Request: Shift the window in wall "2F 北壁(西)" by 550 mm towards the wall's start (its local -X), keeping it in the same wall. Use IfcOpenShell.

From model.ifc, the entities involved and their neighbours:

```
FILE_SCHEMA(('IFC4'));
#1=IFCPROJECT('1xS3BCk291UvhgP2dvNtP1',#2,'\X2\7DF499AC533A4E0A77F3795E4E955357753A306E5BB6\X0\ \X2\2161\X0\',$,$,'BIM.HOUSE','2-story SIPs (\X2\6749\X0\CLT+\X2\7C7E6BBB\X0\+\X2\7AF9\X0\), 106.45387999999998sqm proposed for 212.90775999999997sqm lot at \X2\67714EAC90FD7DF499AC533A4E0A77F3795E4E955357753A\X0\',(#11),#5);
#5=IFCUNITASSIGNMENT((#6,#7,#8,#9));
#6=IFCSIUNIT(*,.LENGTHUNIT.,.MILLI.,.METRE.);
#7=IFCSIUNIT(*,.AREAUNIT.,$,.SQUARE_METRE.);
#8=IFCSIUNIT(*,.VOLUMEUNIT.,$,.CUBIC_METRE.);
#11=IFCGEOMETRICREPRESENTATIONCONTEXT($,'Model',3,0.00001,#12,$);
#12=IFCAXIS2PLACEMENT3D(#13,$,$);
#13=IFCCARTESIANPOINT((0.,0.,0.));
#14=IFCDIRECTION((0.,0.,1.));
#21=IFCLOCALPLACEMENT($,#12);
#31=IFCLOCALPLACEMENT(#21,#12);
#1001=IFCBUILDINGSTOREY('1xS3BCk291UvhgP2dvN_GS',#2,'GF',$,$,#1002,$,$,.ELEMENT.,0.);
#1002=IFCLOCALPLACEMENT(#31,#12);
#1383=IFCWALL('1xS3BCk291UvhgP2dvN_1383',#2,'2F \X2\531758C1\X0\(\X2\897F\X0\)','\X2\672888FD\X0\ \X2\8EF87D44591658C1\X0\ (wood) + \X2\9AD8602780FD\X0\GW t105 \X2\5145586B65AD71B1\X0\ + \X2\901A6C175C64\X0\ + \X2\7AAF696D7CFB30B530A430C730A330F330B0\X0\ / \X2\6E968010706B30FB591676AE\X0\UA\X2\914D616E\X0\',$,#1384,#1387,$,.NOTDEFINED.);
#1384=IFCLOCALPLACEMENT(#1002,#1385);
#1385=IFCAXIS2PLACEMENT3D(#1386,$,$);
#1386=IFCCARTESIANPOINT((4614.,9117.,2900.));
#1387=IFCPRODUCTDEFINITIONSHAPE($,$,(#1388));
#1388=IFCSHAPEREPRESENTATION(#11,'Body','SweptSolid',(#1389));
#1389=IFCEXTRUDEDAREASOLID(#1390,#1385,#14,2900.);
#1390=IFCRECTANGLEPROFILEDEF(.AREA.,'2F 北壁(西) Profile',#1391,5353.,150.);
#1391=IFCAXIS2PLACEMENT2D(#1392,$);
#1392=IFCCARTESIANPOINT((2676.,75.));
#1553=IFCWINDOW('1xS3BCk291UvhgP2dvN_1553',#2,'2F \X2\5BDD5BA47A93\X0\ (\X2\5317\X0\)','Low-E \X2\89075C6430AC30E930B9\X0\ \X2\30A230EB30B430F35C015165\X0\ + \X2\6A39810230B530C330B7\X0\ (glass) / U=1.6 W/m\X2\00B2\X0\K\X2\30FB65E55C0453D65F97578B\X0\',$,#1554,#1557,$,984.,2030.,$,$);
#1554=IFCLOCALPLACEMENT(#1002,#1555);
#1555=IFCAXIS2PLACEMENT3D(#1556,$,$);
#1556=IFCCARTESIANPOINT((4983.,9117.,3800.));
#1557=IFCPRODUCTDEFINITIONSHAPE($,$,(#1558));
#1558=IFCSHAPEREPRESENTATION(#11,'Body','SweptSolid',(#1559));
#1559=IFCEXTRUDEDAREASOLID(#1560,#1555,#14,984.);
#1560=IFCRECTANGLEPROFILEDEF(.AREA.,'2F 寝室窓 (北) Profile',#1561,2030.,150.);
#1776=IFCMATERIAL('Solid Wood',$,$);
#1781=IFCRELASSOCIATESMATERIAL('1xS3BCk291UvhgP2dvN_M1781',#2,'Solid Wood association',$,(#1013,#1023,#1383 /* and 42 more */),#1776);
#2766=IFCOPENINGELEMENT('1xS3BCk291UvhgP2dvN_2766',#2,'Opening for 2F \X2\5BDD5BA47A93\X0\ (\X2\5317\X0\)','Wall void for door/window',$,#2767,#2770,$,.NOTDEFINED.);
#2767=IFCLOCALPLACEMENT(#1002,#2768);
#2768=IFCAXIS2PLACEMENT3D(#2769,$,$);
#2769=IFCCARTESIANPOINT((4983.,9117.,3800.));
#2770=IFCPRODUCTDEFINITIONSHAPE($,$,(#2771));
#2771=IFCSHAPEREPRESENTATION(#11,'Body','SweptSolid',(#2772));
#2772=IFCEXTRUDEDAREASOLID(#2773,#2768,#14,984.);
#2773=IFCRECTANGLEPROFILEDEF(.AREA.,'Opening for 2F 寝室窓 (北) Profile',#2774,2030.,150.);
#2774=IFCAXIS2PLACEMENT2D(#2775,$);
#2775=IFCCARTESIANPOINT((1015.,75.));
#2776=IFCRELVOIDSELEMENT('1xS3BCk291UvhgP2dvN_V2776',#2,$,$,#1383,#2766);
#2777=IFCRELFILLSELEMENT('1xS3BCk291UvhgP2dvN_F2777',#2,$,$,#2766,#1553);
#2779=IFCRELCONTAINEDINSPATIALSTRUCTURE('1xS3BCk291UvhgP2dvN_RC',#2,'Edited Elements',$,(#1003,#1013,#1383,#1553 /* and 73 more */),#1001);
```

```python
import ifcopenshell
import ifcopenshell.api.geometry
import ifcopenshell.util.placement
import ifcopenshell.util.unit

model = ifcopenshell.open("model.ifc")
unit_scale = ifcopenshell.util.unit.calculate_unit_scale(model)

window = model.by_id(1553)
opening = window.FillsVoids[0].RelatingOpeningElement
wall = opening.VoidsElements[0].RelatingBuildingElement

wall_matrix = ifcopenshell.util.placement.get_local_placement(wall.ObjectPlacement)
shift = wall_matrix[:3, 0] * -0.55 / unit_scale
before = ifcopenshell.util.placement.get_local_placement(window.ObjectPlacement)[:3, 3].copy()

# The window is not placed relative to its opening, so move both.
for product in (opening, window):
    matrix = ifcopenshell.util.placement.get_local_placement(product.ObjectPlacement)
    matrix[:3, 3] += shift
    ifcopenshell.api.geometry.edit_object_placement(model, product=product, matrix=matrix, is_si=False)

after = ifcopenshell.util.placement.get_local_placement(window.ObjectPlacement)[:3, 3]
print("window moved by", (after - before).round(3) + 0.0)

model.write("model_edited.ifc")
```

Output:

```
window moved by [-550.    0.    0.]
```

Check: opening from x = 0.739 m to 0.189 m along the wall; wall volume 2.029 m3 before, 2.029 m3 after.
